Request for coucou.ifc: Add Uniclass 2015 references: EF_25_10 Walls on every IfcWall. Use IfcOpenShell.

First a look at what the model holds.

```python
import ifcopenshell

model = ifcopenshell.open("coucou.ifc")
print(model.schema)
print("classifications:", [c.Name for c in model.by_type("IfcClassification")])
for ifc_class in ("IfcDoor", "IfcRoof", "IfcStair", "IfcWall", "IfcWindow"):
    print(ifc_class, len(model.by_type(ifc_class)))
```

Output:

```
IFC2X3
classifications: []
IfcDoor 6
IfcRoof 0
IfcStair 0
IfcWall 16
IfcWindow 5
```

```python
import ifcopenshell
import ifcopenshell.api.classification

model = ifcopenshell.open("coucou.ifc")

# IFC2X3 requires Source and Edition and has no link from the project to the system.
system = model.create_entity("IfcClassification", Source="NBS", Edition="2015", Name="Uniclass 2015")

codes = {
    "IfcWall": ("EF_25_10", "Walls"),
}
for ifc_class, (code, name) in codes.items():
    products = model.by_type(ifc_class)
    ifcopenshell.api.classification.add_reference(
        model, products=products, classification=system, identification=code, name=name
    )
    print(code, len(products))

model.write("coucou_updated.ifc")
```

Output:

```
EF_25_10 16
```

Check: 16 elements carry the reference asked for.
